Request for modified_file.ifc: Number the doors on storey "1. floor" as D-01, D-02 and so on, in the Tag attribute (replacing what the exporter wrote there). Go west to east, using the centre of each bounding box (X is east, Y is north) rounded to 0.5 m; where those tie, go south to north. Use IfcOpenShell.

First a look at what the model holds.

```python
import ifcopenshell
import ifcopenshell.util.element
import ifcopenshell.util.placement

model = ifcopenshell.open("modified_file.ifc")
print(model.schema)
storey = next(s for s in model.by_type("IfcBuildingStorey") if s.Name == "1. floor")
doors = [e for e in ifcopenshell.util.element.get_decomposition(storey) if e.is_a("IfcDoor")]
for e in sorted(doors, key=lambda e: e.id()):
    origin = ifcopenshell.util.placement.get_local_placement(e.ObjectPlacement)[:3, 3]
    print(e.id(), e.Tag, e.Name, origin.round(2) + 0.0, sep=" | ")
```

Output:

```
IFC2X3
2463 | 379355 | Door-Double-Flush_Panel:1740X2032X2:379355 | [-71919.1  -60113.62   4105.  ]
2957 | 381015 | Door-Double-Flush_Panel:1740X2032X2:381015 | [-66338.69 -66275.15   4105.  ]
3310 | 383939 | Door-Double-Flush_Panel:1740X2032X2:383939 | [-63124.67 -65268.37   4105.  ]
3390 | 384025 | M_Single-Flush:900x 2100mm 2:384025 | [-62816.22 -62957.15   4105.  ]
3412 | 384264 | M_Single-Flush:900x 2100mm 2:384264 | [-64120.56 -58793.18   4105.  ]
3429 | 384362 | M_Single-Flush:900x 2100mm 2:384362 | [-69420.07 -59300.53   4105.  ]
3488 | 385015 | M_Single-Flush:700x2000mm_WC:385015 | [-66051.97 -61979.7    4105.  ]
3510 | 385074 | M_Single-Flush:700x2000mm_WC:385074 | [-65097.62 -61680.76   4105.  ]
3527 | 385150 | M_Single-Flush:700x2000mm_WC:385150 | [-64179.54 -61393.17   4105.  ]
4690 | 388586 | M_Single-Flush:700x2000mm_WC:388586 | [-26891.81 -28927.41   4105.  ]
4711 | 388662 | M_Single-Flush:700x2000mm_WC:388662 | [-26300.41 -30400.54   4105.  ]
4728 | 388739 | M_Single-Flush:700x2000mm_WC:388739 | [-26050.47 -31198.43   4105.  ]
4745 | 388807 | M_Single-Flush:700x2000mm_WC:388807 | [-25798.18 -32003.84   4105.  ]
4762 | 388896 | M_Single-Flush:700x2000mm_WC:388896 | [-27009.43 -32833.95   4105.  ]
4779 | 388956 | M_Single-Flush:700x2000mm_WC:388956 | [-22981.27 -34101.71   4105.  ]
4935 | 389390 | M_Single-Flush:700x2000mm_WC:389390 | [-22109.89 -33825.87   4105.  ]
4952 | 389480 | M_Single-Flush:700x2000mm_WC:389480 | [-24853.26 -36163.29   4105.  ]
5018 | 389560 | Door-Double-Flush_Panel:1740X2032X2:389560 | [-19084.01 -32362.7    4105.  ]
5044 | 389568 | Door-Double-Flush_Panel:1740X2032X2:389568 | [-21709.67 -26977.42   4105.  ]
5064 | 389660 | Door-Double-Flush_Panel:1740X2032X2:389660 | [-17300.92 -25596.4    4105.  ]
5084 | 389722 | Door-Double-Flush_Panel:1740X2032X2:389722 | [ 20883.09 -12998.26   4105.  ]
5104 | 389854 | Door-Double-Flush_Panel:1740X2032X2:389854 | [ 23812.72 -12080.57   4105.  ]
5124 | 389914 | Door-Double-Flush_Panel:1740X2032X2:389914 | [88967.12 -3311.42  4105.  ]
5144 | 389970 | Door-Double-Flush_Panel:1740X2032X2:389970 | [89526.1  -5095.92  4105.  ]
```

```python
import ifcopenshell
import ifcopenshell.geom
import ifcopenshell.util.element
import ifcopenshell.util.shape

model = ifcopenshell.open("modified_file.ifc")
settings = ifcopenshell.geom.settings()
settings.set("use-world-coords", True)


def centre(element):
    shape = ifcopenshell.geom.create_shape(settings, element)
    return ifcopenshell.util.shape.get_bbox_centroid(shape.geometry)


storey = next(s for s in model.by_type("IfcBuildingStorey") if s.Name == "1. floor")
doors = [e for e in ifcopenshell.util.element.get_decomposition(storey) if e.is_a("IfcDoor")]

# Insertion points can sit at a corner or the storey origin, so sort by the geometry (in metres).
centres = {e: centre(e) for e in doors}
doors.sort(key=lambda e: (round(centres[e][0] / 0.5), centres[e][1]))

for i, e in enumerate(doors, start=1):
    number = f"D-{i:02d}"
    e.Tag = number
    print(e.id(), number)

model.write("modified_file_v2.ifc")
```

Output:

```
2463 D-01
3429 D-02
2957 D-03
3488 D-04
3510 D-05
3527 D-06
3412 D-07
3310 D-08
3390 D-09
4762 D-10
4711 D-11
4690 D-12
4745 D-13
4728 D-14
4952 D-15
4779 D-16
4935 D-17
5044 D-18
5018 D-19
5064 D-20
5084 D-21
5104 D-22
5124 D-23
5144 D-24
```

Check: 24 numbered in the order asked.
